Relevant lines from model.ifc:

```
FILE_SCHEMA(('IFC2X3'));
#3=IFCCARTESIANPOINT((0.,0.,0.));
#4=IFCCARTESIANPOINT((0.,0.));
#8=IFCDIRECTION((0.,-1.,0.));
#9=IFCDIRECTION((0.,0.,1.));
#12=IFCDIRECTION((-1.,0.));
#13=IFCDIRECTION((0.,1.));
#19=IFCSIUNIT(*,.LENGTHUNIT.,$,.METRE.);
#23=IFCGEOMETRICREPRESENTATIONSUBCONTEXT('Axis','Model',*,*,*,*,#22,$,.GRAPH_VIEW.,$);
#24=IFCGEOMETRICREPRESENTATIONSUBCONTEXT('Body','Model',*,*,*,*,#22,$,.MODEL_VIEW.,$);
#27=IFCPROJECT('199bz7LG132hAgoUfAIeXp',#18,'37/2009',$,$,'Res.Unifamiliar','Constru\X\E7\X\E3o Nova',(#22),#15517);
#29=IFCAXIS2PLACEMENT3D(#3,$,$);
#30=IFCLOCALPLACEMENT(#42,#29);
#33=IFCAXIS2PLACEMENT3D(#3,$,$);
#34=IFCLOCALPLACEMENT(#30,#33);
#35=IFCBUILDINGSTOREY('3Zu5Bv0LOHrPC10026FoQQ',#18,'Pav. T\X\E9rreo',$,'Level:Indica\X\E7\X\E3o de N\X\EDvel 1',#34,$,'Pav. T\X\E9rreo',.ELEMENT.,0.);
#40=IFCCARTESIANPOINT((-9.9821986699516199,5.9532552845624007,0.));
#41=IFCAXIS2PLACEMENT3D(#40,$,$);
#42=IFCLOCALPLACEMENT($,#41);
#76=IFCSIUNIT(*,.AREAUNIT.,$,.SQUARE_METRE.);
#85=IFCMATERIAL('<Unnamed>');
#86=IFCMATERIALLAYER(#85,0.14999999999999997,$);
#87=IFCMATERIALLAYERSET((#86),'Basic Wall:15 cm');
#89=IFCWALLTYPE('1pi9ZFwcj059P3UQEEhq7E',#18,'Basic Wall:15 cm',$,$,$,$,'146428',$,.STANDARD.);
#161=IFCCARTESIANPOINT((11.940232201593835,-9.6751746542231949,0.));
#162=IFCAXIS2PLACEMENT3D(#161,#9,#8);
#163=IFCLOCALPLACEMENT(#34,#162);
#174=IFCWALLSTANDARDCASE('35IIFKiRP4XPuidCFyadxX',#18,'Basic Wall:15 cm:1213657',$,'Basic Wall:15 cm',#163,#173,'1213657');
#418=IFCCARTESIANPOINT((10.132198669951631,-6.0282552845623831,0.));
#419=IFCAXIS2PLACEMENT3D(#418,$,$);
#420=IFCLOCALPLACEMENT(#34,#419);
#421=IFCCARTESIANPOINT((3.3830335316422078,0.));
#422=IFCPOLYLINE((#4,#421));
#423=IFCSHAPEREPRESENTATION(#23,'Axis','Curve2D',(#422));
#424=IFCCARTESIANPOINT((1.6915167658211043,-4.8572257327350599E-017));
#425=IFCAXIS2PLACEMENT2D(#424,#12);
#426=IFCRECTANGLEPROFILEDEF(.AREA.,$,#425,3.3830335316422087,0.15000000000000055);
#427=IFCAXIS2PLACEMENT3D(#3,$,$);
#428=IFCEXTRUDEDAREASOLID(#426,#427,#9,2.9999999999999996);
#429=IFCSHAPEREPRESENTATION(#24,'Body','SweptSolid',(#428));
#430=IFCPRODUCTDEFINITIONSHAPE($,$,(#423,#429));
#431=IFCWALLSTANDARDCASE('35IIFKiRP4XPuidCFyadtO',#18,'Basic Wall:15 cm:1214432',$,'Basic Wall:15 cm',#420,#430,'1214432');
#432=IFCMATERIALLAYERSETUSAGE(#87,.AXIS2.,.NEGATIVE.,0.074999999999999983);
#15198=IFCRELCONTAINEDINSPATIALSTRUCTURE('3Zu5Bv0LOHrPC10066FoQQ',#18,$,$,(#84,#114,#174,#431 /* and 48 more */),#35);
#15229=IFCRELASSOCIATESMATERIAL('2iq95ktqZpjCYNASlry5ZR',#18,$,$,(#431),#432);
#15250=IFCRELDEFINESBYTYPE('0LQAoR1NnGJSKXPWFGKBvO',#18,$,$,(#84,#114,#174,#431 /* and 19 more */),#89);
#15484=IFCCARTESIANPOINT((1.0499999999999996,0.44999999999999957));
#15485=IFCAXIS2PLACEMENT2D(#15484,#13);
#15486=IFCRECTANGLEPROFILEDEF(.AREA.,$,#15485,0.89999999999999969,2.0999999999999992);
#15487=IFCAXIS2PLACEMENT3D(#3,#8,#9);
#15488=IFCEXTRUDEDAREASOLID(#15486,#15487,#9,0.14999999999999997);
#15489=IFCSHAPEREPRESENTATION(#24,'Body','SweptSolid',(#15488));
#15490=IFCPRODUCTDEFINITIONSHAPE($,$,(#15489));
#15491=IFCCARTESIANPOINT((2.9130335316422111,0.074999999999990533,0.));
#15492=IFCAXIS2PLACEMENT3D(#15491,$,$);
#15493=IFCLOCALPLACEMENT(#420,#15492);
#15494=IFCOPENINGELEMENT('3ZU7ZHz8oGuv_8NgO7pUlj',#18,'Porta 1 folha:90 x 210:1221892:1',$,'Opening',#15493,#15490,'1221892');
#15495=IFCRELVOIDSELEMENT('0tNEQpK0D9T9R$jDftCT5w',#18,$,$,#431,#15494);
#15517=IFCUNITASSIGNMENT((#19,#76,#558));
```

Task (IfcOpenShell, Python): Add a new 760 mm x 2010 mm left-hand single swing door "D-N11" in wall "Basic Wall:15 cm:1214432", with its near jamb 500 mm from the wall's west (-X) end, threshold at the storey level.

```python
import numpy as np
import ifcopenshell
import ifcopenshell.api.feature
import ifcopenshell.api.geometry
import ifcopenshell.api.root
import ifcopenshell.api.spatial
import ifcopenshell.api.type
import ifcopenshell.geom
import ifcopenshell.util.element
import ifcopenshell.util.placement
import ifcopenshell.util.representation
import ifcopenshell.util.shape
import ifcopenshell.util.unit

model = ifcopenshell.open("model.ifc")
unit_scale = ifcopenshell.util.unit.calculate_unit_scale(model)
settings = ifcopenshell.geom.settings()


def volume(element):
    """Net volume in cubic metres, openings subtracted."""
    shape = ifcopenshell.geom.create_shape(settings, element)
    return ifcopenshell.util.shape.get_volume(shape.geometry)


wall = model.by_guid("35IIFKiRP4XPuidCFyadtO")
storey = ifcopenshell.util.element.get_container(wall, ifc_class="IfcBuildingStorey")
context = ifcopenshell.util.representation.get_context(model, "Model", "Body", "MODEL_VIEW")
before = volume(wall)

width, height, from_end, sill = 0.76, 2.01, 0.5, 0.0  # metres

# The wall runs along its own X axis, and the end named is its -X end.
wall_shape = ifcopenshell.geom.create_shape(settings, wall)
x, y, z = ifcopenshell.util.shape.get_vertices(wall_shape.geometry).T
start = x.min() + from_end
face, thickness = float(y.min()), float(y.max() - y.min())
wall_matrix = ifcopenshell.util.placement.get_local_placement(wall.ObjectPlacement)
level = ifcopenshell.util.placement.get_local_placement(storey.ObjectPlacement)[2, 3]


def in_wall(x, y):
    """Placement at x, y metres in the wall's axes, at sill height."""
    matrix = wall_matrix.copy()
    matrix[:, 3] = wall_matrix @ np.array([x / unit_scale, y / unit_scale, 0.0, 1.0])
    matrix[2, 3] = level + sill / unit_scale
    return matrix


# Opening: a box that overshoots both wall faces by 50 mm.
opening = ifcopenshell.api.root.create_entity(model, ifc_class="IfcOpeningElement")
box = ifcopenshell.api.geometry.add_wall_representation(
    model, context=context, length=width, height=height, thickness=thickness + 0.1
)
ifcopenshell.api.geometry.assign_representation(model, product=opening, representation=box)
ifcopenshell.api.geometry.edit_object_placement(model, product=opening, matrix=in_wall(start, face - 0.05), is_si=False)
ifcopenshell.api.feature.add_feature(model, feature=opening, element=wall)

door = ifcopenshell.api.root.create_entity(model, ifc_class="IfcDoor", name="D-N11")
door.OverallWidth, door.OverallHeight = width / unit_scale, height / unit_scale
body = ifcopenshell.api.geometry.add_door_representation(
    model,
    context=context,
    overall_width=door.OverallWidth,
    overall_height=door.OverallHeight,
    operation_type="SINGLE_SWING_LEFT",
    lining_properties={"LiningDepth": thickness / unit_scale, "ThresholdDepth": thickness / unit_scale},
)
ifcopenshell.api.geometry.assign_representation(model, product=door, representation=body)
ifcopenshell.api.spatial.assign_container(model, products=[door], relating_structure=storey)
fills = ifcopenshell.api.feature.add_filling(model, opening=opening, element=door)
fills.OwnerHistory = door.OwnerHistory  # required in IFC2X3

# IFC2X3 keeps the operation on the door style.
style = ifcopenshell.api.root.create_entity(model, ifc_class="IfcDoorStyle", name="D-N11")
style.OperationType, style.ConstructionType = "SINGLE_SWING_LEFT", "NOTDEFINED"
style.ParameterTakesPrecedence = style.Sizeable = False
ifcopenshell.api.type.assign_type(model, related_objects=[door], relating_type=style)

# The lining spans the wall, so the door starts at the wall face.
ifcopenshell.api.geometry.edit_object_placement(model, product=door, matrix=in_wall(start, face), is_si=False)

after = volume(wall)

print(f"wall volume {before:.3f} -> {after:.3f} m3")

model.write("model_updated.ifc")
```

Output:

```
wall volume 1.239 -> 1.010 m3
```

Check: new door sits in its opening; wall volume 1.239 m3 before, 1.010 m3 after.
